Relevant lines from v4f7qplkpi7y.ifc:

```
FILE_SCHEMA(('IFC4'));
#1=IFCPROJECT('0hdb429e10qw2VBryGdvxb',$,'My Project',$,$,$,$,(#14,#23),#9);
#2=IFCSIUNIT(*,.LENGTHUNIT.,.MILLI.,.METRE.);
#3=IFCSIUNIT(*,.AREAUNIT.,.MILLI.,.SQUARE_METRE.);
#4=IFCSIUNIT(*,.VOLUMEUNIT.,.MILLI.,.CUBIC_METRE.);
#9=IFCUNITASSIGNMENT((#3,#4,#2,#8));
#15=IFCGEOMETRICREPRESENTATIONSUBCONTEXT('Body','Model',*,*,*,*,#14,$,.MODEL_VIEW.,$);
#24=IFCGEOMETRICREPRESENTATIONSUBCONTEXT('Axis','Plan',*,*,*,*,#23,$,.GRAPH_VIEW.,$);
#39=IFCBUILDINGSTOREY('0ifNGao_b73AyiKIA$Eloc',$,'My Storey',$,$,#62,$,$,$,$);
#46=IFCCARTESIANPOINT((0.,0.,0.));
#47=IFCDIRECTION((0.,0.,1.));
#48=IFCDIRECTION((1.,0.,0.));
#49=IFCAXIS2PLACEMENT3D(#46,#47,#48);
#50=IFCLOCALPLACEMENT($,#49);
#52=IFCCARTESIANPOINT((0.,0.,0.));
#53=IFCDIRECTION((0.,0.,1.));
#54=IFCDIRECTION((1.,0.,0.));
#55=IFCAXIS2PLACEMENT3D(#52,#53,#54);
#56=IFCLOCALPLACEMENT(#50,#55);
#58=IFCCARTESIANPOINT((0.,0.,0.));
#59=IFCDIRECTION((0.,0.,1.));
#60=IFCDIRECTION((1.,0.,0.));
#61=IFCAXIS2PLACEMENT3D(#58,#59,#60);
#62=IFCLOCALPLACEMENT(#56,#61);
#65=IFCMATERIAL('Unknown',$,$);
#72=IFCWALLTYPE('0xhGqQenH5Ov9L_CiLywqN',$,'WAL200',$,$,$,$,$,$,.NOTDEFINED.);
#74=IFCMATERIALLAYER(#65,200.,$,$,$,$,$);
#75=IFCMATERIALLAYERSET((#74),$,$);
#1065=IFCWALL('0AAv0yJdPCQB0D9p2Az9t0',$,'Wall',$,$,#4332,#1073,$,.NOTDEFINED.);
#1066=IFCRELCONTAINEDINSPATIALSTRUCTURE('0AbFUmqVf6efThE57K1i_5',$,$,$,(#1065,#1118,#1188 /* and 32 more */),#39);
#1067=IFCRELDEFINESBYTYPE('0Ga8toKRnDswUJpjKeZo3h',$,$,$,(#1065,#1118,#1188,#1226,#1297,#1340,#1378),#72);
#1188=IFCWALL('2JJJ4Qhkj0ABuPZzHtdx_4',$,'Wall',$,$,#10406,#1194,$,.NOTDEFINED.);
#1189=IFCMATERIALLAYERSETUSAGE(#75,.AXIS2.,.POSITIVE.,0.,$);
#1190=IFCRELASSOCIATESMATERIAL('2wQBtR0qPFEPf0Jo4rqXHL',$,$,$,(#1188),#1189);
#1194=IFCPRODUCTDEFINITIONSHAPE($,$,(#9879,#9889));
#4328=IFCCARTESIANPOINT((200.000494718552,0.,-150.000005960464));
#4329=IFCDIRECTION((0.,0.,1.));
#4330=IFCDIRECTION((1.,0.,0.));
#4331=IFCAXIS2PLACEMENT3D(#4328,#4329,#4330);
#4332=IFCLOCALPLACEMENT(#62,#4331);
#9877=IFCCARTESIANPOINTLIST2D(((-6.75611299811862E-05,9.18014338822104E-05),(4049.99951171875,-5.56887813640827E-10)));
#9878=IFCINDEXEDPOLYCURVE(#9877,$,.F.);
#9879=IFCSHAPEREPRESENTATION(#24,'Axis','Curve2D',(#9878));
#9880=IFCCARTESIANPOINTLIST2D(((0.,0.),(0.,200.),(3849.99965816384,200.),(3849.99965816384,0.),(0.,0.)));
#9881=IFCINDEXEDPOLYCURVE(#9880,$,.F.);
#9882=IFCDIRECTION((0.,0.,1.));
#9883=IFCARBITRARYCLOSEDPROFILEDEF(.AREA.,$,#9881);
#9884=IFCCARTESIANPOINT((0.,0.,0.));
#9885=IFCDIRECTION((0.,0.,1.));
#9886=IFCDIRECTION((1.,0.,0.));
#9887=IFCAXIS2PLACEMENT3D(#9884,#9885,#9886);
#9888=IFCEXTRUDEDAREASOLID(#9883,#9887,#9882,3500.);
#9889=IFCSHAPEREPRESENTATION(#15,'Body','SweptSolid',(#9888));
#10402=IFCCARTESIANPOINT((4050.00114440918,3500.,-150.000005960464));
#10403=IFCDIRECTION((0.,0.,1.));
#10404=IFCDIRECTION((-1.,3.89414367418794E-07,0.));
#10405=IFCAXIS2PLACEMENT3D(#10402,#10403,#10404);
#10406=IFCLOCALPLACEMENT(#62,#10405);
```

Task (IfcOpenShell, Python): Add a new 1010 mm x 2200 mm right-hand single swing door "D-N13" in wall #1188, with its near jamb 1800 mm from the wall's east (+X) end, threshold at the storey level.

```python
import numpy as np
import ifcopenshell
import ifcopenshell.api.feature
import ifcopenshell.api.geometry
import ifcopenshell.api.root
import ifcopenshell.api.spatial
import ifcopenshell.geom
import ifcopenshell.util.element
import ifcopenshell.util.placement
import ifcopenshell.util.representation
import ifcopenshell.util.shape
import ifcopenshell.util.unit

model = ifcopenshell.open("v4f7qplkpi7y.ifc")
unit_scale = ifcopenshell.util.unit.calculate_unit_scale(model)
settings = ifcopenshell.geom.settings()


def volume(element):
    """Net volume in cubic metres, openings subtracted."""
    shape = ifcopenshell.geom.create_shape(settings, element)
    return ifcopenshell.util.shape.get_volume(shape.geometry)


wall = model.by_guid("2JJJ4Qhkj0ABuPZzHtdx_4")
storey = ifcopenshell.util.element.get_container(wall, ifc_class="IfcBuildingStorey")
context = ifcopenshell.util.representation.get_context(model, "Model", "Body", "MODEL_VIEW")
before = volume(wall)

width, height, from_end, sill = 1.01, 2.2, 1.8, 0.0  # metres

# The wall runs along its own X axis, and the end named is its -X end.
wall_shape = ifcopenshell.geom.create_shape(settings, wall)
x, y, z = ifcopenshell.util.shape.get_vertices(wall_shape.geometry).T
start = x.min() + from_end
face, thickness = float(y.min()), float(y.max() - y.min())
wall_matrix = ifcopenshell.util.placement.get_local_placement(wall.ObjectPlacement)
level = ifcopenshell.util.placement.get_local_placement(storey.ObjectPlacement)[2, 3]


def in_wall(x, y):
    """Placement at x, y metres in the wall's axes, at sill height."""
    matrix = wall_matrix.copy()
    matrix[:, 3] = wall_matrix @ np.array([x / unit_scale, y / unit_scale, 0.0, 1.0])
    matrix[2, 3] = level + sill / unit_scale
    return matrix


# Opening: a box that overshoots both wall faces by 50 mm.
opening = ifcopenshell.api.root.create_entity(model, ifc_class="IfcOpeningElement", predefined_type="OPENING")
box = ifcopenshell.api.geometry.add_wall_representation(
    model, context=context, length=width, height=height, thickness=thickness + 0.1
)
ifcopenshell.api.geometry.assign_representation(model, product=opening, representation=box)
ifcopenshell.api.geometry.edit_object_placement(model, product=opening, matrix=in_wall(start, face - 0.05), is_si=False)
ifcopenshell.api.feature.add_feature(model, feature=opening, element=wall)

door = ifcopenshell.api.root.create_entity(model, ifc_class="IfcDoor", name="D-N13", predefined_type="DOOR")
door.OverallWidth, door.OverallHeight = width / unit_scale, height / unit_scale
door.OperationType = "SINGLE_SWING_RIGHT"
body = ifcopenshell.api.geometry.add_door_representation(
    model,
    context=context,
    overall_width=door.OverallWidth,
    overall_height=door.OverallHeight,
    operation_type="SINGLE_SWING_RIGHT",
    lining_properties={"LiningDepth": thickness / unit_scale, "ThresholdDepth": thickness / unit_scale},
)
ifcopenshell.api.geometry.assign_representation(model, product=door, representation=body)
ifcopenshell.api.spatial.assign_container(model, products=[door], relating_structure=storey)
ifcopenshell.api.feature.add_filling(model, opening=opening, element=door)

# The lining spans the wall, so the door starts at the wall face.
ifcopenshell.api.geometry.edit_object_placement(model, product=door, matrix=in_wall(start, face), is_si=False)

after = volume(wall)

print(f"wall volume {before:.3f} -> {after:.3f} m3")

model.write("v4f7qplkpi7y_edited.ifc")
```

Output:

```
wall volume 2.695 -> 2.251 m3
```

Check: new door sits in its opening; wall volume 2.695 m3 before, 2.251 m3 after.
